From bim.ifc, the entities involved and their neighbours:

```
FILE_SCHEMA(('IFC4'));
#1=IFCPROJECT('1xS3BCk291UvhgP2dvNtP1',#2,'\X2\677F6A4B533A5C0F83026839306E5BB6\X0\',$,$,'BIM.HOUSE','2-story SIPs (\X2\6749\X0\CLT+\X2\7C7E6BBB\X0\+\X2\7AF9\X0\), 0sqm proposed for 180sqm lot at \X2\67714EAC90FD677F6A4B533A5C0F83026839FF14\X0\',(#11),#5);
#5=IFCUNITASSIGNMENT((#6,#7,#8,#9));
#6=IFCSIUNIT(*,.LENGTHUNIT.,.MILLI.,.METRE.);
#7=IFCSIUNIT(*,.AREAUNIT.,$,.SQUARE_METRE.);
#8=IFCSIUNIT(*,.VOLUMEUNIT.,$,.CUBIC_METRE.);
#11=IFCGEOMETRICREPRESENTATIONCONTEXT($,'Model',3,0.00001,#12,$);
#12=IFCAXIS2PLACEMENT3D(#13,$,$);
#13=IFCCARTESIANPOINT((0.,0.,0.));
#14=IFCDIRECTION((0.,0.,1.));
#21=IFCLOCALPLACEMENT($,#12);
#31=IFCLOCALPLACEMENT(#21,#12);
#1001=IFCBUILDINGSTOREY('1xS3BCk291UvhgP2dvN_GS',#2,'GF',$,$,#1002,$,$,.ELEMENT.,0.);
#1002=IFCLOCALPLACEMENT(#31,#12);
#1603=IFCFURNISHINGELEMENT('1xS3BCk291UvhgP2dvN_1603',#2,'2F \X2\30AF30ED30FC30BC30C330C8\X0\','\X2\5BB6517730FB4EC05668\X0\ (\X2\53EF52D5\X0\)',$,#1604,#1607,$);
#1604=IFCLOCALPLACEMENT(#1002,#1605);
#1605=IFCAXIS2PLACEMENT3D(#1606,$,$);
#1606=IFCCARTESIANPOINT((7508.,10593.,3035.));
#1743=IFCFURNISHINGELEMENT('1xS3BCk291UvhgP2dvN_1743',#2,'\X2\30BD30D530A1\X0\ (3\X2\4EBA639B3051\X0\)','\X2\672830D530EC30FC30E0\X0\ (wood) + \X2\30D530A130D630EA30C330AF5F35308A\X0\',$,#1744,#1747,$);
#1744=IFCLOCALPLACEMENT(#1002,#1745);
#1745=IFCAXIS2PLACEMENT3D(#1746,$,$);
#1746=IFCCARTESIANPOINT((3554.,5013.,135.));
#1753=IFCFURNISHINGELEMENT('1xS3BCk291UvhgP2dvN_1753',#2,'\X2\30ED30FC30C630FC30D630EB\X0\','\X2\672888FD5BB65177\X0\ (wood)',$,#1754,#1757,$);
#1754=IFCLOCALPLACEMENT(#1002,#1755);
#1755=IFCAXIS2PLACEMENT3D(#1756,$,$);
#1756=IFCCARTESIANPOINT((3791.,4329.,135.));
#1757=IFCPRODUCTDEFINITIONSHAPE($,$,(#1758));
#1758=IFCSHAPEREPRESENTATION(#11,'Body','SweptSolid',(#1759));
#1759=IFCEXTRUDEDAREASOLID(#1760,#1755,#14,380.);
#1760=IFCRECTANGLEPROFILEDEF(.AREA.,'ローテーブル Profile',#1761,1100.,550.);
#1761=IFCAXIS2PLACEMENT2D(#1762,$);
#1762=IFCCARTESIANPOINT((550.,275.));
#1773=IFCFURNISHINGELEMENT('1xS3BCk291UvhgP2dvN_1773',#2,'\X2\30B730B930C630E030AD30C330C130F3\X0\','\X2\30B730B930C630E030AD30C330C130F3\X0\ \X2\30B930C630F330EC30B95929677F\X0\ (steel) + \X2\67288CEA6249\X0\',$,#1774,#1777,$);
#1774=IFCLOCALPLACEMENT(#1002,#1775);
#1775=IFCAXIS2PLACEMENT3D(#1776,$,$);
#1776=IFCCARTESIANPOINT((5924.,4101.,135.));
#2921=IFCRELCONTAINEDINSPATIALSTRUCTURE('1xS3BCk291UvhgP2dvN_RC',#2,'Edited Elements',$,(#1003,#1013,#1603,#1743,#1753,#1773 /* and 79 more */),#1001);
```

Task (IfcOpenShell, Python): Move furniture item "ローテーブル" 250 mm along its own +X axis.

```python
import ifcopenshell
import ifcopenshell.api.geometry
import ifcopenshell.util.placement

model = ifcopenshell.open("bim.ifc")

item = model.by_guid("1xS3BCk291UvhgP2dvN_1753")
matrix = ifcopenshell.util.placement.get_local_placement(item.ObjectPlacement)
matrix[:3, 3] += matrix[:3, 0] * 250.0
ifcopenshell.api.geometry.edit_object_placement(model, product=item, matrix=matrix, is_si=False)

print(ifcopenshell.util.placement.get_local_placement(item.ObjectPlacement).round(3) + 0.0)

model.write("bim_updated.ifc")
```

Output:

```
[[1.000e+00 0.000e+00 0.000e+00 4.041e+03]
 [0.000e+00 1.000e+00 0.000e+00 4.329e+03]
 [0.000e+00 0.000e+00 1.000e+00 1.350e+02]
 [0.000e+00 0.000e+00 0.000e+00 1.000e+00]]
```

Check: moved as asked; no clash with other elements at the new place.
